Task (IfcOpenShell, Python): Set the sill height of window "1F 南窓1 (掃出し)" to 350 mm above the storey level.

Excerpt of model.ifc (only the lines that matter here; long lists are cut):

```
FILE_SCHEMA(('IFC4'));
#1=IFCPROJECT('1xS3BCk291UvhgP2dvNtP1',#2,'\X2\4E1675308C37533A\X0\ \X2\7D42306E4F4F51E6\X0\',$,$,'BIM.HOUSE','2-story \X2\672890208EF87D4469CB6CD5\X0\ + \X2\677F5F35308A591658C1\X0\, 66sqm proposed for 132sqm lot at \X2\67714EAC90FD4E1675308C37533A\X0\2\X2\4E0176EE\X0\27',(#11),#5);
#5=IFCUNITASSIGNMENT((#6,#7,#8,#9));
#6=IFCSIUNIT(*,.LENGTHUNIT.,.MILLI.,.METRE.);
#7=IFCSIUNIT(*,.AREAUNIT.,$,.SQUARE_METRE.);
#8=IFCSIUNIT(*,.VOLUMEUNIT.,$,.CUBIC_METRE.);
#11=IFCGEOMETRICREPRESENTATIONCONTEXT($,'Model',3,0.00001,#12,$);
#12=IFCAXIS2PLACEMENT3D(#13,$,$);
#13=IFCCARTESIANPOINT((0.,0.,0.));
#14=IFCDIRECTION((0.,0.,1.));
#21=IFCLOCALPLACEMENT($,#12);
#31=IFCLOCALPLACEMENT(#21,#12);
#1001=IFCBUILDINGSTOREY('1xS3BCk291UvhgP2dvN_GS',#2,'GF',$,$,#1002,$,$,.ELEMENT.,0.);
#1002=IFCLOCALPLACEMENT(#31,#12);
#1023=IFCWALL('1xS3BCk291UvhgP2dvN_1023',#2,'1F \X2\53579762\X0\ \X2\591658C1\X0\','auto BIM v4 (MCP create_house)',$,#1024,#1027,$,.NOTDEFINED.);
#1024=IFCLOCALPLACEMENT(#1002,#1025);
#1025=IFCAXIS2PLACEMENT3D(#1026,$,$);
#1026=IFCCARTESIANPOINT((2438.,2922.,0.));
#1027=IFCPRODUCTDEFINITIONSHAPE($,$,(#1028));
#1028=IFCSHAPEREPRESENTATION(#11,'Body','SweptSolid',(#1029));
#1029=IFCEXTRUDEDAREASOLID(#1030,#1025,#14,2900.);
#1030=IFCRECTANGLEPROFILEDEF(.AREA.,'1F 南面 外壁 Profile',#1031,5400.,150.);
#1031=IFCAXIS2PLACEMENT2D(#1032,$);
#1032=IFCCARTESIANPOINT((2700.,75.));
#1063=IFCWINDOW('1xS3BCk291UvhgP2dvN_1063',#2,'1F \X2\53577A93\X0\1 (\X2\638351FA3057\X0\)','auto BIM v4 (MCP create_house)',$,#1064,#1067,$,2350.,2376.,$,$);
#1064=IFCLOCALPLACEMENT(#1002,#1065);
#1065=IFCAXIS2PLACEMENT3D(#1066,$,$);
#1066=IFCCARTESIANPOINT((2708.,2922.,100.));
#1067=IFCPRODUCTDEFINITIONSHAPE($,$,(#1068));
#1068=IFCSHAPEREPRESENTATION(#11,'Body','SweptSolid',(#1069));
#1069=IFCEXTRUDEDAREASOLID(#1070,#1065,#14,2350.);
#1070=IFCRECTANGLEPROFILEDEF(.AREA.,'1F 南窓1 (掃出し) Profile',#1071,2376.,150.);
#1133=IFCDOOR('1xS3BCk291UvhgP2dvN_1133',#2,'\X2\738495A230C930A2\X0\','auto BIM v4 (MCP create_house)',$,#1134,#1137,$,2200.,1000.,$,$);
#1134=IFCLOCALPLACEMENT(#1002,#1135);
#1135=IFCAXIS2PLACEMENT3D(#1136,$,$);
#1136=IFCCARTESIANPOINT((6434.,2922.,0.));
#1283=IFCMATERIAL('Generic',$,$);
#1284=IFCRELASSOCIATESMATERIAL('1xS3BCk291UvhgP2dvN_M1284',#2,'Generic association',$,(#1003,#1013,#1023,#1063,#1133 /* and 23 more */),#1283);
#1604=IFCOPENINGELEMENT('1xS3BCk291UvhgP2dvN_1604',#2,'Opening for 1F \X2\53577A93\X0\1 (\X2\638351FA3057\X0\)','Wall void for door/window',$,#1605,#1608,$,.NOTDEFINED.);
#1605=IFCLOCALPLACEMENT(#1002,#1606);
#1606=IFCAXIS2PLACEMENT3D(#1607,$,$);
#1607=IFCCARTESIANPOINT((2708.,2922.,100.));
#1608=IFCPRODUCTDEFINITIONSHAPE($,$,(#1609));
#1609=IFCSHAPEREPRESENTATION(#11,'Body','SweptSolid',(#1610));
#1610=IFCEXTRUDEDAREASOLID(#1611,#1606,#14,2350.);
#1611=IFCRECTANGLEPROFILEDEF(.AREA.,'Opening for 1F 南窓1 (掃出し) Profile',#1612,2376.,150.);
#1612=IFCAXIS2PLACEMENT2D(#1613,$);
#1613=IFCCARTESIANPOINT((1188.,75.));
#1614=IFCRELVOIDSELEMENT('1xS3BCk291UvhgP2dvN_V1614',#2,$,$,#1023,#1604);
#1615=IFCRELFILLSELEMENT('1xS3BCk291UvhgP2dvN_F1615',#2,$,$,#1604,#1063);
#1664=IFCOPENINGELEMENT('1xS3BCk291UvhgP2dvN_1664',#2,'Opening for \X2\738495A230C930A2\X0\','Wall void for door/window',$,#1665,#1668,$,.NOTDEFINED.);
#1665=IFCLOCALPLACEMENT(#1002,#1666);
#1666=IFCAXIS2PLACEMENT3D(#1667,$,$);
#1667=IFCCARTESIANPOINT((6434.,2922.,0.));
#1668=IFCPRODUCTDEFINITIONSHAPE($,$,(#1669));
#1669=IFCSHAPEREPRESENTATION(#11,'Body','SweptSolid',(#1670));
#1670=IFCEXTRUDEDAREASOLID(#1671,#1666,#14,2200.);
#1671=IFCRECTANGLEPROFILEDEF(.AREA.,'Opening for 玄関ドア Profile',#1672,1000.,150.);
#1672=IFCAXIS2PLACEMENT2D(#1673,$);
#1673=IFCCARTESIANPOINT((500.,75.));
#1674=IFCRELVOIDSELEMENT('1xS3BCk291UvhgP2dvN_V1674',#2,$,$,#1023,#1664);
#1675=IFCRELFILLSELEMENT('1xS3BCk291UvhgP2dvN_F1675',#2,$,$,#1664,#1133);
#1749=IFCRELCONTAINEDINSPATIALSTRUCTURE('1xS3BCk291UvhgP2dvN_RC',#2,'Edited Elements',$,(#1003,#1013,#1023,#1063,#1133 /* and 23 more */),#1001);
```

```python
import numpy as np
import ifcopenshell
import ifcopenshell.api.geometry
import ifcopenshell.geom
import ifcopenshell.util.element
import ifcopenshell.util.placement
import ifcopenshell.util.shape
import ifcopenshell.util.unit

model = ifcopenshell.open("model.ifc")
unit_scale = ifcopenshell.util.unit.calculate_unit_scale(model)

window = model.by_guid("1xS3BCk291UvhgP2dvN_1063")
opening = window.FillsVoids[0].RelatingOpeningElement
storey = ifcopenshell.util.element.get_container(window, ifc_class="IfcBuildingStorey")
level = ifcopenshell.util.placement.get_local_placement(storey.ObjectPlacement)[2, 3]

# The opening's origin need not be at the sill, so measure its lowest point.
shape = ifcopenshell.geom.create_shape(ifcopenshell.geom.settings(), opening)
bottom = ifcopenshell.util.shape.get_shape_bottom_elevation(shape, shape.geometry) / unit_scale
dz = level + 0.35 / unit_scale - bottom

shift = np.array([0.0, 0.0, dz])
# The window is not placed relative to its opening, so move both.
for product in (opening, window):
    matrix = ifcopenshell.util.placement.get_local_placement(product.ObjectPlacement)
    matrix[:3, 3] += shift
    ifcopenshell.api.geometry.edit_object_placement(model, product=product, matrix=matrix, is_si=False)

print(f"moved by {dz * unit_scale:+.3f} m")

model.write("model_rev.ifc")
```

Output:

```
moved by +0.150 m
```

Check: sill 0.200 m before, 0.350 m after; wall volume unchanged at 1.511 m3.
